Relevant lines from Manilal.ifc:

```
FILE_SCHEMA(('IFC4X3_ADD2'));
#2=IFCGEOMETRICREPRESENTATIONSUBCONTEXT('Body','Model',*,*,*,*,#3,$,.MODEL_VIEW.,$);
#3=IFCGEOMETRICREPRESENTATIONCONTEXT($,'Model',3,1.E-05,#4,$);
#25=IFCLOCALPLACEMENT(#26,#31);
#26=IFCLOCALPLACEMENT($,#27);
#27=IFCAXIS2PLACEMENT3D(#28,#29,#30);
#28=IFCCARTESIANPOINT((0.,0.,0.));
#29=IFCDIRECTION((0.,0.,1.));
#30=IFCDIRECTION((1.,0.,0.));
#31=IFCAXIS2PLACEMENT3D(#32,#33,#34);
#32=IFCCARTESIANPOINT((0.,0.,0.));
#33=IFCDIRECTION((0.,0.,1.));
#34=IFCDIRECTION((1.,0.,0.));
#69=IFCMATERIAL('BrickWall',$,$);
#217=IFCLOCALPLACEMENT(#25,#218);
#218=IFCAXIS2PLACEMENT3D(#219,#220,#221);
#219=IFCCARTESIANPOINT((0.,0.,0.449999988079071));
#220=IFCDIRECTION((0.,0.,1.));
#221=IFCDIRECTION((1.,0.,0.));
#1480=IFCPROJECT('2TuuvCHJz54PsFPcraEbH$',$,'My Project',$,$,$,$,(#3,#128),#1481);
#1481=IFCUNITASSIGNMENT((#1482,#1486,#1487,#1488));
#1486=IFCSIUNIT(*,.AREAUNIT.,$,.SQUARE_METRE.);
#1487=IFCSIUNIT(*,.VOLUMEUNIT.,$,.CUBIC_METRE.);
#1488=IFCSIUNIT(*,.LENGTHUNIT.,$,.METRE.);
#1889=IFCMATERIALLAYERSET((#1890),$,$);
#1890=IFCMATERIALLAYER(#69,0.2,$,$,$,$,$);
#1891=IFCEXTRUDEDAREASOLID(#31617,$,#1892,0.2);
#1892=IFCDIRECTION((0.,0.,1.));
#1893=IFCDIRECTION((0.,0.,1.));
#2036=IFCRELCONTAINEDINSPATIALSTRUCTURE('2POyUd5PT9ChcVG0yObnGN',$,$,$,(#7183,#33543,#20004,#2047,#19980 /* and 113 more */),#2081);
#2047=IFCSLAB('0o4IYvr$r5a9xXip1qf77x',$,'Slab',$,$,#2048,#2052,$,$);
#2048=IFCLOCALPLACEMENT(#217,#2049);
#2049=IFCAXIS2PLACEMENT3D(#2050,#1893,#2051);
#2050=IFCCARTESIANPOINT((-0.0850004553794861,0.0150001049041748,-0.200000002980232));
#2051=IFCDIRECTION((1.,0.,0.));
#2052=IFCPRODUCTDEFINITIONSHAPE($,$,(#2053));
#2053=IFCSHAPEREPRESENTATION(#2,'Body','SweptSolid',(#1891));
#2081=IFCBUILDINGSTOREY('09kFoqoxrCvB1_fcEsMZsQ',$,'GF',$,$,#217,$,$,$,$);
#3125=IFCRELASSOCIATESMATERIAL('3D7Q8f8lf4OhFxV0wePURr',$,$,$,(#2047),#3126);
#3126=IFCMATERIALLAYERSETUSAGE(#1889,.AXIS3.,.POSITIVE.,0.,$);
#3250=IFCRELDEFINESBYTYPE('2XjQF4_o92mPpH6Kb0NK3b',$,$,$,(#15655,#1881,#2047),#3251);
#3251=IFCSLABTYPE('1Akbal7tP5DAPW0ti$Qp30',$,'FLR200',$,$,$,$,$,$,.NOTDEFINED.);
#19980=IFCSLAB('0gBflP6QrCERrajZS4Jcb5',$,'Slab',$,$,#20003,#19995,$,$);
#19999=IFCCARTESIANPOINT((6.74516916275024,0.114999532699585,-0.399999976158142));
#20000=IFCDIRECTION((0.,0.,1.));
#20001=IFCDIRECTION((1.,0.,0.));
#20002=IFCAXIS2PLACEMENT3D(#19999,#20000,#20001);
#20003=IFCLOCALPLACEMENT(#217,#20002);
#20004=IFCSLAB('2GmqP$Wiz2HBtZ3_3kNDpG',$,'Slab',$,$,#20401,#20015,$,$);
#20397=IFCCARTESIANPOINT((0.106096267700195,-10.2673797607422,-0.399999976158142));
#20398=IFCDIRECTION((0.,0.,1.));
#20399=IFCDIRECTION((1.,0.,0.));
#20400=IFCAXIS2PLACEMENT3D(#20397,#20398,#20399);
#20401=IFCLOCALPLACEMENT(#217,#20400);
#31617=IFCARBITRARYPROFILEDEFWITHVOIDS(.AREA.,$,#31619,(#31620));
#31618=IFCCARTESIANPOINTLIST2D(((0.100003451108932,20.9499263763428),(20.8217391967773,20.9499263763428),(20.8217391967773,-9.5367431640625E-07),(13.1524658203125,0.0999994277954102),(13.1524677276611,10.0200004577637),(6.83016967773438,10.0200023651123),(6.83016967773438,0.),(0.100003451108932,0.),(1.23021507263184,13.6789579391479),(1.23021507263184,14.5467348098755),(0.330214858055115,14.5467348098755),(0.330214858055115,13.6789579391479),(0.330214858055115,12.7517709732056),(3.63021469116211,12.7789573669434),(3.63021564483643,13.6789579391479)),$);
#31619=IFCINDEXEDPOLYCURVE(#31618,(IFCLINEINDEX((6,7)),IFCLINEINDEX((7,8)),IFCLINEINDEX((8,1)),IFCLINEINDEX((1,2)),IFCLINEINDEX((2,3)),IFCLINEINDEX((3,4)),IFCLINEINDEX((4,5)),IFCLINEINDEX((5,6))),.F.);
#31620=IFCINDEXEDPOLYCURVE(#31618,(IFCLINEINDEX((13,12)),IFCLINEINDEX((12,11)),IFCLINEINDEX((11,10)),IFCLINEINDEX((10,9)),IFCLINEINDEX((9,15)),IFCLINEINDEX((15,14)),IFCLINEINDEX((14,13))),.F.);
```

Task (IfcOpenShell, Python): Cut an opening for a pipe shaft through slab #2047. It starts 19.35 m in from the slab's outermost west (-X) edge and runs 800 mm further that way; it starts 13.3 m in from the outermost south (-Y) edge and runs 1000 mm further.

```python
import numpy as np
import ifcopenshell
import ifcopenshell.api.feature
import ifcopenshell.api.geometry
import ifcopenshell.api.root
import ifcopenshell.geom
import ifcopenshell.util.placement
import ifcopenshell.util.representation
import ifcopenshell.util.shape
import ifcopenshell.util.unit

model = ifcopenshell.open("Manilal.ifc")
unit_scale = ifcopenshell.util.unit.calculate_unit_scale(model)
settings = ifcopenshell.geom.settings()


def volume(element):
    """Net volume in cubic metres, openings subtracted."""
    shape = ifcopenshell.geom.create_shape(settings, element)
    return ifcopenshell.util.shape.get_volume(shape.geometry)


slab = model.by_guid("0o4IYvr$r5a9xXip1qf77x")
before = volume(slab)

# Extent in the slab's own axes, in metres. The edges named are its -X and -Y sides.
slab_shape = ifcopenshell.geom.create_shape(settings, slab)
vertices = ifcopenshell.util.shape.get_vertices(slab_shape.geometry)
x_min, y_min, bottom = vertices.min(axis=0)
top = vertices[:, 2].max()

opening = ifcopenshell.api.root.create_entity(model, ifc_class="IfcOpeningElement", name="Pipe shaft opening", predefined_type="OPENING")
context = ifcopenshell.util.representation.get_context(model, "Model", "Body", "MODEL_VIEW")
width, depth = 0.8, 1
outline = [(0.0, 0.0), (width, 0.0), (width, depth), (0.0, depth), (0.0, 0.0)]
# Overshoot both faces by 50 mm so the cut is clean.
shape = ifcopenshell.api.geometry.add_slab_representation(
    model, context=context, depth=top - bottom + 0.1, polyline=outline
)
ifcopenshell.api.geometry.assign_representation(model, product=opening, representation=shape)

matrix = ifcopenshell.util.placement.get_local_placement(slab.ObjectPlacement)
matrix[:, 3] = matrix @ np.append(np.array([x_min + 19.35, y_min + 13.3, bottom - 0.05]) / unit_scale, 1.0)
ifcopenshell.api.geometry.edit_object_placement(model, product=opening, matrix=matrix, is_si=False)
ifcopenshell.api.feature.add_feature(model, feature=opening, element=slab)

after = volume(slab)

print(f"slab volume {before:.3f} -> {after:.3f} m3")

model.write("Manilal-out.ifc")
```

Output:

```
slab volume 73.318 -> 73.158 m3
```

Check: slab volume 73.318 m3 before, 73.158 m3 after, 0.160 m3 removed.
